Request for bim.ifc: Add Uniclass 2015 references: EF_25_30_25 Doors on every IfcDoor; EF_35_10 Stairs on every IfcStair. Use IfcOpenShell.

First a look at what the model holds.

```python
import ifcopenshell

model = ifcopenshell.open("bim.ifc")
print(model.schema)
print("classifications:", [c.Name for c in model.by_type("IfcClassification")])
for ifc_class in ("IfcDoor", "IfcRoof", "IfcStair", "IfcWall", "IfcWindow"):
    print(ifc_class, len(model.by_type(ifc_class)))
```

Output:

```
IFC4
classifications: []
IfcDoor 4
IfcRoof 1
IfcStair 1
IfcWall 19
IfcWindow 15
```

```python
import ifcopenshell
import ifcopenshell.api.classification

model = ifcopenshell.open("bim.ifc")

system = ifcopenshell.api.classification.add_classification(model, classification="Uniclass 2015")

codes = {
    "IfcDoor": ("EF_25_30_25", "Doors"),
    "IfcStair": ("EF_35_10", "Stairs"),
}
for ifc_class, (code, name) in codes.items():
    products = model.by_type(ifc_class)
    ifcopenshell.api.classification.add_reference(
        model, products=products, classification=system, identification=code, name=name
    )
    print(code, len(products))

model.write("bim_v2.ifc")
```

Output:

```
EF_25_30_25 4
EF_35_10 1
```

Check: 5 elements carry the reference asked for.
